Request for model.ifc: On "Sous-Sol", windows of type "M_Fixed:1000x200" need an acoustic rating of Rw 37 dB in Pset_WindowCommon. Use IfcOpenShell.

First a look at what the model holds.

```python
import ifcopenshell
import ifcopenshell.util.element

model = ifcopenshell.open("model.ifc")
print(model.schema)
storey = next(s for s in model.by_type("IfcBuildingStorey") if s.Name == "Sous-Sol")
windows = [e for e in ifcopenshell.util.element.get_decomposition(storey) if e.is_a("IfcWindow")]
seen = {}
for e in windows:
    element_type = ifcopenshell.util.element.get_type(e)
    key = (element_type.Name if element_type != e and element_type else None, ifcopenshell.util.element.get_pset(e, "Pset_WindowCommon", "AcousticRating"))
    seen[key] = seen.get(key, 0) + 1
for (name, value), count in sorted(seen.items(), key=str):
    print(count, "x", name, "|", value)
```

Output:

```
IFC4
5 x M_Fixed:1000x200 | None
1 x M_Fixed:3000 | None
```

```python
import ifcopenshell
import ifcopenshell.api.pset
import ifcopenshell.util.element

model = ifcopenshell.open("model.ifc")

storey = next(s for s in model.by_type("IfcBuildingStorey") if s.Name == "Sous-Sol")
windows = [e for e in ifcopenshell.util.element.get_decomposition(storey) if e.is_a("IfcWindow")]

count = 0
for e in windows:
    element_type = ifcopenshell.util.element.get_type(e)
    if element_type in (None, e) or element_type.Name != "M_Fixed:1000x200":
        continue
    # add_pset returns the element's existing set when there is one.
    pset = ifcopenshell.api.pset.add_pset(model, product=e, name="Pset_WindowCommon")
    ifcopenshell.api.pset.edit_pset(model, pset=pset, properties={"AcousticRating": "Rw 37 dB"})
    count += 1

print(count, "windows updated")

model.write("model-out.ifc")
```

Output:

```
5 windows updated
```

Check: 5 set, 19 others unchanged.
